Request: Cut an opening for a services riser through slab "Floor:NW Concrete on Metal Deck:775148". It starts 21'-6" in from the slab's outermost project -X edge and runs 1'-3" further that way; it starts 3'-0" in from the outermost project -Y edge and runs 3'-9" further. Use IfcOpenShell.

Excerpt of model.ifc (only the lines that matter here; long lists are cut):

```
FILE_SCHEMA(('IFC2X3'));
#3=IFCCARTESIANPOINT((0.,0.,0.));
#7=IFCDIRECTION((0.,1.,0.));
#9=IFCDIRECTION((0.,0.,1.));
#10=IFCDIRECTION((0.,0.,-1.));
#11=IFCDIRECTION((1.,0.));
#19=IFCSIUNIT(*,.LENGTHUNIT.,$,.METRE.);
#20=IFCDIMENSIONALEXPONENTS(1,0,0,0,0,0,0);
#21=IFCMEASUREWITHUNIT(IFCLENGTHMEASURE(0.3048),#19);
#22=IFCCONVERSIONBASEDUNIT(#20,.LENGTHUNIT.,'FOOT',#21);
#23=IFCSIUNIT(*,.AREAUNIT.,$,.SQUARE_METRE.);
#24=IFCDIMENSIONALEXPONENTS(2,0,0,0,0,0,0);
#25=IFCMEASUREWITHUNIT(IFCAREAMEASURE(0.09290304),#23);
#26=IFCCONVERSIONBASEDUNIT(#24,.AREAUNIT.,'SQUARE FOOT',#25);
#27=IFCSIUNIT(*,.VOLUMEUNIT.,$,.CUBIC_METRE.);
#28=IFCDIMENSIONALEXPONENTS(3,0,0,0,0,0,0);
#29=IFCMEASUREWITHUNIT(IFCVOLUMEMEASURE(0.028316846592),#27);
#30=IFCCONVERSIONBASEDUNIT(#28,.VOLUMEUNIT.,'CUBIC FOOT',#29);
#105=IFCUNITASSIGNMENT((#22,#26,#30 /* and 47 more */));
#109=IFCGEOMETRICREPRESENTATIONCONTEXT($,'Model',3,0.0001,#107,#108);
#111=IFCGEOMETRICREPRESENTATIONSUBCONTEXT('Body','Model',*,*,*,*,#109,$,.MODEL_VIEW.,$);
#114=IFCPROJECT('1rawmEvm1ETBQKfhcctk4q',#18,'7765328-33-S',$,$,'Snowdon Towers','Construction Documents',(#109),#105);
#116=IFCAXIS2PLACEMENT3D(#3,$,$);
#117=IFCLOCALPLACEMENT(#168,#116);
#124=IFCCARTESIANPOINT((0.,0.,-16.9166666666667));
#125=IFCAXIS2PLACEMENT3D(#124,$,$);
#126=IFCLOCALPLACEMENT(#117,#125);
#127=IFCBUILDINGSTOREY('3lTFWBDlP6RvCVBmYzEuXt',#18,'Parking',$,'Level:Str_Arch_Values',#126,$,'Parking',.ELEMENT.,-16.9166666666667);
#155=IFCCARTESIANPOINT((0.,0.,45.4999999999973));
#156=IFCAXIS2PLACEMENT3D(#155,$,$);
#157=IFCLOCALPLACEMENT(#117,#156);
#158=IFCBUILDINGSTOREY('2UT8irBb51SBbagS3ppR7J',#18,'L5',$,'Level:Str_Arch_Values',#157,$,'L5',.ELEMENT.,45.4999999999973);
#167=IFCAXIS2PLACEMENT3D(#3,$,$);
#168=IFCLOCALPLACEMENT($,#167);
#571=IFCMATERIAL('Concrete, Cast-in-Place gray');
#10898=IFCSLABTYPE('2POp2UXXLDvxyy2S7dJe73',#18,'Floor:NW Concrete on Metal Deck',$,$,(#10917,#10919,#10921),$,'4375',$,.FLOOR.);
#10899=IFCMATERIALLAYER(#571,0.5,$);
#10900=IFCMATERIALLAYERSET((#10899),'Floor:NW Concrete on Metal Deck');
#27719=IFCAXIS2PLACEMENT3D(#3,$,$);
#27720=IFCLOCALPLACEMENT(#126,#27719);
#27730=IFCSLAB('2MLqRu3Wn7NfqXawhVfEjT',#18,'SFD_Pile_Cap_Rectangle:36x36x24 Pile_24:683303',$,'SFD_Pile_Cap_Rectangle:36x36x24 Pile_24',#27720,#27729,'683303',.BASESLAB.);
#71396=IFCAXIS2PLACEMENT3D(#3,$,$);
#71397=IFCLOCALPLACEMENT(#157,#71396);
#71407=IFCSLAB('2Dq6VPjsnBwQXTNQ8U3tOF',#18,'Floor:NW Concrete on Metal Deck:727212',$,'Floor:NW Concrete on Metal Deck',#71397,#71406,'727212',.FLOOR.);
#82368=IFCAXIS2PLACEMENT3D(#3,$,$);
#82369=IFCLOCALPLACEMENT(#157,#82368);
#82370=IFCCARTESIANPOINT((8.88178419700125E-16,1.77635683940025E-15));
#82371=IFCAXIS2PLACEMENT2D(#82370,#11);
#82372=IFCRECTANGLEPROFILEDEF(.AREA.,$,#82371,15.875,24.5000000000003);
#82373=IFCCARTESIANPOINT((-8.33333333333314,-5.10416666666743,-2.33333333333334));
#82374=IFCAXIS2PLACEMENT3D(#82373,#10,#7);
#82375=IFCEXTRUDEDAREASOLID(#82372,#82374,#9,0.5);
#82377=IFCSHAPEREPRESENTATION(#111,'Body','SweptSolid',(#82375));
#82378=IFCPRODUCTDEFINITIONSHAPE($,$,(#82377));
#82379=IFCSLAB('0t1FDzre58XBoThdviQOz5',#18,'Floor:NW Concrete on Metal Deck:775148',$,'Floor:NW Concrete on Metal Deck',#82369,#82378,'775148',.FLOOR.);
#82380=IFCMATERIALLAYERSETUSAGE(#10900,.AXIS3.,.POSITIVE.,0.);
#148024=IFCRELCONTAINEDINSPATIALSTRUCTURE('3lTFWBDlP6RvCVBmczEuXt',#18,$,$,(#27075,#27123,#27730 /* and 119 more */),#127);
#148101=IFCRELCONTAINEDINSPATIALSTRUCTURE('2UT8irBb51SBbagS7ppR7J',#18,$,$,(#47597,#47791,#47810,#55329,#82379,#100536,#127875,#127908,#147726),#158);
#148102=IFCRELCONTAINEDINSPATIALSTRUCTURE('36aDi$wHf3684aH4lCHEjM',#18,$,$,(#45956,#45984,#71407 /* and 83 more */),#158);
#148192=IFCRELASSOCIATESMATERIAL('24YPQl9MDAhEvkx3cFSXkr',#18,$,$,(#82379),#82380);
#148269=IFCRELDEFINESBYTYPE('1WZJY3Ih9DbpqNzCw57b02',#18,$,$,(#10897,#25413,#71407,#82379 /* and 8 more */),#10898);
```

```python
import numpy as np
import ifcopenshell
import ifcopenshell.api.feature
import ifcopenshell.api.geometry
import ifcopenshell.api.root
import ifcopenshell.geom
import ifcopenshell.util.placement
import ifcopenshell.util.representation
import ifcopenshell.util.shape
import ifcopenshell.util.unit

model = ifcopenshell.open("model.ifc")
unit_scale = ifcopenshell.util.unit.calculate_unit_scale(model)
settings = ifcopenshell.geom.settings()


def volume(element):
    """Net volume in cubic metres, openings subtracted."""
    shape = ifcopenshell.geom.create_shape(settings, element)
    return ifcopenshell.util.shape.get_volume(shape.geometry)


slab = model.by_id(82379)
before = volume(slab)

# Extent in the slab's own axes, in metres. The edges named are its -X and -Y sides.
slab_shape = ifcopenshell.geom.create_shape(settings, slab)
vertices = ifcopenshell.util.shape.get_vertices(slab_shape.geometry)
x_min, y_min, bottom = vertices.min(axis=0)
top = vertices[:, 2].max()

opening = ifcopenshell.api.root.create_entity(model, ifc_class="IfcOpeningElement", name="Services riser opening")
context = ifcopenshell.util.representation.get_context(model, "Model", "Body", "MODEL_VIEW")
width, depth = 0.381, 1.143
outline = [(0.0, 0.0), (width, 0.0), (width, depth), (0.0, depth), (0.0, 0.0)]
# Overshoot both faces by 50 mm so the cut is clean.
shape = ifcopenshell.api.geometry.add_slab_representation(
    model, context=context, depth=top - bottom + 0.1, polyline=outline
)
ifcopenshell.api.geometry.assign_representation(model, product=opening, representation=shape)

matrix = ifcopenshell.util.placement.get_local_placement(slab.ObjectPlacement)
matrix[:, 3] = matrix @ np.append(np.array([x_min + 6.5532, y_min + 0.9144, bottom - 0.05]) / unit_scale, 1.0)
ifcopenshell.api.geometry.edit_object_placement(model, product=opening, matrix=matrix, is_si=False)
ifcopenshell.api.feature.add_feature(model, feature=opening, element=slab)

after = volume(slab)

print(f"slab volume {before:.3f} -> {after:.3f} m3")

model.write("model-out.ifc")
```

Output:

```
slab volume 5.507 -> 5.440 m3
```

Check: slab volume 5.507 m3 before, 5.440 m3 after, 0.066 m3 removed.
